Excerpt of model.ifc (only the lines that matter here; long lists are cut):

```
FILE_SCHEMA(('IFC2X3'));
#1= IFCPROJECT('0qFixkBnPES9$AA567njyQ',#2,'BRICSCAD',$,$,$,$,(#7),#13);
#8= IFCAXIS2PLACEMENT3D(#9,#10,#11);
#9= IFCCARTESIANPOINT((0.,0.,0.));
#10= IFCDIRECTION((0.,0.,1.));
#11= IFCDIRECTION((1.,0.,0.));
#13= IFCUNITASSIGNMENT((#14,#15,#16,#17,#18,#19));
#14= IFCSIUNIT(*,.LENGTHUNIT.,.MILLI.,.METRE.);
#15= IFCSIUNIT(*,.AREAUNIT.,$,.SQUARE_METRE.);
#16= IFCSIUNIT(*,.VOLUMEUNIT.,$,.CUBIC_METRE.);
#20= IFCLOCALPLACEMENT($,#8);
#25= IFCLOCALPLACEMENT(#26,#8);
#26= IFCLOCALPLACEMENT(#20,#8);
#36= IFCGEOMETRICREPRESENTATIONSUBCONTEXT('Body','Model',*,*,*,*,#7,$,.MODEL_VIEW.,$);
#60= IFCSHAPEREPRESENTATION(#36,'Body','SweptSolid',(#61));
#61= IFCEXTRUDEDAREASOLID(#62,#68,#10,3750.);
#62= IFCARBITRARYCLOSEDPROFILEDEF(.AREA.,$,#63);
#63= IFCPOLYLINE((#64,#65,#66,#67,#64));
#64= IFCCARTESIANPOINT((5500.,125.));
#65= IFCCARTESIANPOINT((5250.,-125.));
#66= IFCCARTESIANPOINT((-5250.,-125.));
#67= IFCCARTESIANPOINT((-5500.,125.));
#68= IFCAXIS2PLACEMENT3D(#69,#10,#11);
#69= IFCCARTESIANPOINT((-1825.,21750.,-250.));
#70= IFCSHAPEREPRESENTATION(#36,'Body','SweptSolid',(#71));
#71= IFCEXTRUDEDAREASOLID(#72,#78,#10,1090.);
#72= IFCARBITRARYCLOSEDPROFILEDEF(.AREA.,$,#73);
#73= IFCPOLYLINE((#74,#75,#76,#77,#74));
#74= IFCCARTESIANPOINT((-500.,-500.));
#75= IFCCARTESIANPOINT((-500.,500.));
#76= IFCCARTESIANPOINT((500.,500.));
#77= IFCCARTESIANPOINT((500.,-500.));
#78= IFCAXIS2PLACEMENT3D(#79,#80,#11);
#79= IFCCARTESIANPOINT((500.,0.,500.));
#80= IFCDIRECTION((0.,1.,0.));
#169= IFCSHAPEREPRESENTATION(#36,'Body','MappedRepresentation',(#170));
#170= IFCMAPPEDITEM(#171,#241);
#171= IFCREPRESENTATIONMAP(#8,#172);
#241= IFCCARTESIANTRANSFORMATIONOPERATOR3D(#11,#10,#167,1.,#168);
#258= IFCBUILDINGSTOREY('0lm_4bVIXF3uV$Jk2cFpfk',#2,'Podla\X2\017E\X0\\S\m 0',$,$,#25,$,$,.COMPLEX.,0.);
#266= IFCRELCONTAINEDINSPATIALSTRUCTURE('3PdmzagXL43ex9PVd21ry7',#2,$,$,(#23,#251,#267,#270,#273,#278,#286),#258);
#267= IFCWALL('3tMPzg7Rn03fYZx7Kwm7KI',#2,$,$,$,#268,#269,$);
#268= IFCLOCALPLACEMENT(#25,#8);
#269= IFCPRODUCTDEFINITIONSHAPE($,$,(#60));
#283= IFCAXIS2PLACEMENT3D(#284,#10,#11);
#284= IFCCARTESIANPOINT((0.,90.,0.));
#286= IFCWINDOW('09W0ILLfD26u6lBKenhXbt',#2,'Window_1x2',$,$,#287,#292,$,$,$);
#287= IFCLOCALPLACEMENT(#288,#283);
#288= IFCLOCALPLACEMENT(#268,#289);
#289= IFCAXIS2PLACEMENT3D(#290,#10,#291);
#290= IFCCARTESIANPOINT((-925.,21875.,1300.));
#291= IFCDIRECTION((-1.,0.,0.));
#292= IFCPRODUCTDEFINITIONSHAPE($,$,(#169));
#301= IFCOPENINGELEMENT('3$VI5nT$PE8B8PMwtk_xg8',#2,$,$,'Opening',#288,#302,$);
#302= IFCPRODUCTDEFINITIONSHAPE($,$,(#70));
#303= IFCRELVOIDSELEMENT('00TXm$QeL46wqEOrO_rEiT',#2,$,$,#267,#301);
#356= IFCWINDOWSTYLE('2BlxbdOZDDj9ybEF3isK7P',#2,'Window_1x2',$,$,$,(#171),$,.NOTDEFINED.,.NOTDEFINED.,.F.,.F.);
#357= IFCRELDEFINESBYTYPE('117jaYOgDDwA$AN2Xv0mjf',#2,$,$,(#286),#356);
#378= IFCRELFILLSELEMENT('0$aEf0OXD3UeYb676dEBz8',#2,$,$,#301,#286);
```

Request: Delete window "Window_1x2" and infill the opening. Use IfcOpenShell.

```python
import ifcopenshell
import ifcopenshell.api.feature
import ifcopenshell.api.root
import ifcopenshell.geom
import ifcopenshell.util.shape

model = ifcopenshell.open("model.ifc")
settings = ifcopenshell.geom.settings()


def volume(element):
    """Net volume in cubic metres, openings subtracted."""
    shape = ifcopenshell.geom.create_shape(settings, element)
    return ifcopenshell.util.shape.get_volume(shape.geometry)


window = model.by_id(286)
opening = window.FillsVoids[0].RelatingOpeningElement
wall = opening.VoidsElements[0].RelatingBuildingElement
before = volume(wall)

ifcopenshell.api.root.remove_product(model, product=window)
ifcopenshell.api.feature.remove_feature(model, feature=opening)

after = volume(wall)

print(f"wall volume {before:.3f} -> {after:.3f} m3")

model.write("model_edited.ifc")
```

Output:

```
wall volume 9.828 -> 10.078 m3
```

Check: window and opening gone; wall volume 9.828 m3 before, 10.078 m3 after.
